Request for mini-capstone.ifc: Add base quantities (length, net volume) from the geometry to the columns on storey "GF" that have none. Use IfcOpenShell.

First a look at what the model holds.

```python
import ifcopenshell
import ifcopenshell.util.element
import ifcopenshell.util.unit

model = ifcopenshell.open("mini-capstone.ifc")
print(model.schema)
for unit_type in ("LENGTHUNIT", "AREAUNIT", "VOLUMEUNIT"):
    print(unit_type, ifcopenshell.util.unit.calculate_unit_scale(model, unit_type))
storey = next(s for s in model.by_type("IfcBuildingStorey") if s.Name == "GF")
columns = [e for e in ifcopenshell.util.element.get_decomposition(storey) if e.is_a("IfcColumn")]
for e in sorted(columns, key=lambda e: e.id()):
    print(e.id(), e.is_a(), e.Name, list(ifcopenshell.util.element.get_psets(e, qtos_only=True)), sep=" | ")
```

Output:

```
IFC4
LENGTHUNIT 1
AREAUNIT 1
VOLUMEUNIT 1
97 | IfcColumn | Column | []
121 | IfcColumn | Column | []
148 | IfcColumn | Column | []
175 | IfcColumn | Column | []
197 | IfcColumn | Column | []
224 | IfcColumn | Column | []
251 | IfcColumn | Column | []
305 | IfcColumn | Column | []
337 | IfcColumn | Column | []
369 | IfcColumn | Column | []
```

```python
import ifcopenshell
import ifcopenshell.api.pset
import ifcopenshell.geom
import ifcopenshell.util.element
import ifcopenshell.util.shape
import ifcopenshell.util.unit

model = ifcopenshell.open("mini-capstone.ifc")
unit_scale = ifcopenshell.util.unit.calculate_unit_scale(model)
volume_scale = ifcopenshell.util.unit.calculate_unit_scale(model, "VOLUMEUNIT")
settings = ifcopenshell.geom.settings()

storey = next(s for s in model.by_type("IfcBuildingStorey") if s.Name == "GF")
columns = [e for e in ifcopenshell.util.element.get_decomposition(storey) if e.is_a("IfcColumn")]

for e in sorted(columns, key=lambda e: e.id()):
    if ifcopenshell.util.element.get_psets(e, qtos_only=True, should_inherit=False):
        continue
    # Geometry comes back in metres, in the element's own axes.
    shape = ifcopenshell.geom.create_shape(settings, e)
    values = {
        "Length": ifcopenshell.util.shape.get_z(shape.geometry) / unit_scale,
        "NetVolume": ifcopenshell.util.shape.get_volume(shape.geometry) / volume_scale,
    }
    qto = ifcopenshell.api.pset.add_qto(model, product=e, name="Qto_ColumnBaseQuantities")
    ifcopenshell.api.pset.edit_qto(model, qto=qto, properties=values)
    print(e.id(), {k: round(v, 3) for k, v in values.items()})

model.write("mini-capstone_rev.ifc")
```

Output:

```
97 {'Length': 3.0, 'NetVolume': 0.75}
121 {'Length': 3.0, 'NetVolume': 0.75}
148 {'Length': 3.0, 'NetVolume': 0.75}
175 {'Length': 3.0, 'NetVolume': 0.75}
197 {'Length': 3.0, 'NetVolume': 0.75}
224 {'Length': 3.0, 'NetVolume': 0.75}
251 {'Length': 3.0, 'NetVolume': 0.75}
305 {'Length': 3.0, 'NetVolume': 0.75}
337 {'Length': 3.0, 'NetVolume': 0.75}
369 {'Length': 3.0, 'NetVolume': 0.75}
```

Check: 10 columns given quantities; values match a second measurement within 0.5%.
